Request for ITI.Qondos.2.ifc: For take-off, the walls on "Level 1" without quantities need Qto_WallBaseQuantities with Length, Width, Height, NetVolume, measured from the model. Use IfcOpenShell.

First a look at what the model holds.

```python
import ifcopenshell
import ifcopenshell.util.element
import ifcopenshell.util.unit

model = ifcopenshell.open("ITI.Qondos.2.ifc")
print(model.schema)
for unit_type in ("LENGTHUNIT", "AREAUNIT", "VOLUMEUNIT"):
    print(unit_type, ifcopenshell.util.unit.calculate_unit_scale(model, unit_type))
storey = next(s for s in model.by_type("IfcBuildingStorey") if s.Name == "Level 1")
walls = [e for e in ifcopenshell.util.element.get_decomposition(storey) if e.is_a("IfcWall")]
for e in sorted(walls, key=lambda e: e.id()):
    print(e.id(), e.is_a(), e.Name, list(ifcopenshell.util.element.get_psets(e, qtos_only=True)), sep=" | ")
```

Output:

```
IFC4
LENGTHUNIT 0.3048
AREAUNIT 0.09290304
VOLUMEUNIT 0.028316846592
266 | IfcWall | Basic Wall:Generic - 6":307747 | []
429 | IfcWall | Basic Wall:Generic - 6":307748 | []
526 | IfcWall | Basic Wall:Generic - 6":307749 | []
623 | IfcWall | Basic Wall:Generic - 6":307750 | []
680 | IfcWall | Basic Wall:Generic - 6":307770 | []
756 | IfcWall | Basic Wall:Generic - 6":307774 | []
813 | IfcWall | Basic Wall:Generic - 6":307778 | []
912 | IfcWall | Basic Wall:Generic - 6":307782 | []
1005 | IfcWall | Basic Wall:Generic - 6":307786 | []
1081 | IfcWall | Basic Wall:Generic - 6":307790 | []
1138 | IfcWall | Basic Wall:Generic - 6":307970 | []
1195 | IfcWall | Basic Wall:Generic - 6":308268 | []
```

```python
import ifcopenshell
import ifcopenshell.api.pset
import ifcopenshell.geom
import ifcopenshell.util.element
import ifcopenshell.util.shape
import ifcopenshell.util.unit

model = ifcopenshell.open("ITI.Qondos.2.ifc")
unit_scale = ifcopenshell.util.unit.calculate_unit_scale(model)
volume_scale = ifcopenshell.util.unit.calculate_unit_scale(model, "VOLUMEUNIT")
settings = ifcopenshell.geom.settings()

storey = next(s for s in model.by_type("IfcBuildingStorey") if s.Name == "Level 1")
walls = [e for e in ifcopenshell.util.element.get_decomposition(storey) if e.is_a("IfcWall")]

for e in sorted(walls, key=lambda e: e.id()):
    if ifcopenshell.util.element.get_psets(e, qtos_only=True, should_inherit=False):
        continue
    # Geometry comes back in metres, in the element's own axes.
    shape = ifcopenshell.geom.create_shape(settings, e)
    values = {
        "Length": ifcopenshell.util.shape.get_x(shape.geometry) / unit_scale,
        "Width": ifcopenshell.util.shape.get_y(shape.geometry) / unit_scale,
        "Height": ifcopenshell.util.shape.get_z(shape.geometry) / unit_scale,
        "NetVolume": ifcopenshell.util.shape.get_volume(shape.geometry) / volume_scale,
    }
    qto = ifcopenshell.api.pset.add_qto(model, product=e, name="Qto_WallBaseQuantities")
    ifcopenshell.api.pset.edit_qto(model, qto=qto, properties=values)
    print(e.id(), {k: round(v, 3) for k, v in values.items()})

model.write("ITI.Qondos.2_updated.ifc")
```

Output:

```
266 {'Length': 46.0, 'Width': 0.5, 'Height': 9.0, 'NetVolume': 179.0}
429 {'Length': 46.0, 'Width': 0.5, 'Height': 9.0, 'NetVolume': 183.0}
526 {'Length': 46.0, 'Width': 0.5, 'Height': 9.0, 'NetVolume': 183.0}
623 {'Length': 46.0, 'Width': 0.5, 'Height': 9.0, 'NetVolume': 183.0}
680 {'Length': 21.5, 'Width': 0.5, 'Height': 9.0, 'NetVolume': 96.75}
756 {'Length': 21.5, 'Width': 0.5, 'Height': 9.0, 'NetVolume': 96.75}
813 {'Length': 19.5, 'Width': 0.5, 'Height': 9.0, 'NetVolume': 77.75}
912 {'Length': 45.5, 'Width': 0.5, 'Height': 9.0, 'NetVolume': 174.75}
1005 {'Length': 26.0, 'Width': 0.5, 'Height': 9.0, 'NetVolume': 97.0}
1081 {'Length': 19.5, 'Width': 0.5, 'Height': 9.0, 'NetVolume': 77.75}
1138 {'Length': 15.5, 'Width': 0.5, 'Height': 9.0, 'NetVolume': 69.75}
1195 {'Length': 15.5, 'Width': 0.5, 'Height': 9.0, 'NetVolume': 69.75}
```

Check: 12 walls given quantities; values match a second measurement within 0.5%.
